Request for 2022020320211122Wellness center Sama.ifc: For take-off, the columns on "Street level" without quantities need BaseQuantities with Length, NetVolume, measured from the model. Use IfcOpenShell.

First a look at what the model holds.

```python
import ifcopenshell
import ifcopenshell.util.element
import ifcopenshell.util.unit

model = ifcopenshell.open("2022020320211122Wellness center Sama.ifc")
print(model.schema)
for unit_type in ("LENGTHUNIT", "AREAUNIT", "VOLUMEUNIT"):
    print(unit_type, ifcopenshell.util.unit.calculate_unit_scale(model, unit_type))
storey = next(s for s in model.by_type("IfcBuildingStorey") if s.Name == "Street level")
columns = [e for e in ifcopenshell.util.element.get_decomposition(storey) if e.is_a("IfcColumn")]
for e in sorted(columns, key=lambda e: e.id()):
    print(e.id(), e.is_a(), e.Name, list(ifcopenshell.util.element.get_psets(e, qtos_only=True)), sep=" | ")
```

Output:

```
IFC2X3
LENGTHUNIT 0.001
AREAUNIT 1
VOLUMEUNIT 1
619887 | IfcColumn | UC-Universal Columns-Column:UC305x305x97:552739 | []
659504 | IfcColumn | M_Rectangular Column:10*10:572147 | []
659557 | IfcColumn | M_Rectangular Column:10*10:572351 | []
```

```python
import ifcopenshell
import ifcopenshell.api.pset
import ifcopenshell.geom
import ifcopenshell.util.element
import ifcopenshell.util.shape
import ifcopenshell.util.unit

model = ifcopenshell.open("2022020320211122Wellness center Sama.ifc")
unit_scale = ifcopenshell.util.unit.calculate_unit_scale(model)
volume_scale = ifcopenshell.util.unit.calculate_unit_scale(model, "VOLUMEUNIT")
settings = ifcopenshell.geom.settings()

storey = next(s for s in model.by_type("IfcBuildingStorey") if s.Name == "Street level")
columns = [e for e in ifcopenshell.util.element.get_decomposition(storey) if e.is_a("IfcColumn")]

for e in sorted(columns, key=lambda e: e.id()):
    if ifcopenshell.util.element.get_psets(e, qtos_only=True, should_inherit=False):
        continue
    # Geometry comes back in metres, in the element's own axes.
    shape = ifcopenshell.geom.create_shape(settings, e)
    values = {
        "Length": ifcopenshell.util.shape.get_z(shape.geometry) / unit_scale,
        "NetVolume": ifcopenshell.util.shape.get_volume(shape.geometry) / volume_scale,
    }
    qto = ifcopenshell.api.pset.add_qto(model, product=e, name="BaseQuantities")
    ifcopenshell.api.pset.edit_qto(model, qto=qto, properties=values)
    print(e.id(), {k: round(v, 3) for k, v in values.items()})

model.write("2022020320211122Wellness center Sama_v2.ifc")
```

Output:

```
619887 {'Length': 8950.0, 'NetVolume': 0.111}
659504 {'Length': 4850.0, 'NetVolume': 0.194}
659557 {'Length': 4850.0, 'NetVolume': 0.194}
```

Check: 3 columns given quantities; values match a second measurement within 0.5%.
